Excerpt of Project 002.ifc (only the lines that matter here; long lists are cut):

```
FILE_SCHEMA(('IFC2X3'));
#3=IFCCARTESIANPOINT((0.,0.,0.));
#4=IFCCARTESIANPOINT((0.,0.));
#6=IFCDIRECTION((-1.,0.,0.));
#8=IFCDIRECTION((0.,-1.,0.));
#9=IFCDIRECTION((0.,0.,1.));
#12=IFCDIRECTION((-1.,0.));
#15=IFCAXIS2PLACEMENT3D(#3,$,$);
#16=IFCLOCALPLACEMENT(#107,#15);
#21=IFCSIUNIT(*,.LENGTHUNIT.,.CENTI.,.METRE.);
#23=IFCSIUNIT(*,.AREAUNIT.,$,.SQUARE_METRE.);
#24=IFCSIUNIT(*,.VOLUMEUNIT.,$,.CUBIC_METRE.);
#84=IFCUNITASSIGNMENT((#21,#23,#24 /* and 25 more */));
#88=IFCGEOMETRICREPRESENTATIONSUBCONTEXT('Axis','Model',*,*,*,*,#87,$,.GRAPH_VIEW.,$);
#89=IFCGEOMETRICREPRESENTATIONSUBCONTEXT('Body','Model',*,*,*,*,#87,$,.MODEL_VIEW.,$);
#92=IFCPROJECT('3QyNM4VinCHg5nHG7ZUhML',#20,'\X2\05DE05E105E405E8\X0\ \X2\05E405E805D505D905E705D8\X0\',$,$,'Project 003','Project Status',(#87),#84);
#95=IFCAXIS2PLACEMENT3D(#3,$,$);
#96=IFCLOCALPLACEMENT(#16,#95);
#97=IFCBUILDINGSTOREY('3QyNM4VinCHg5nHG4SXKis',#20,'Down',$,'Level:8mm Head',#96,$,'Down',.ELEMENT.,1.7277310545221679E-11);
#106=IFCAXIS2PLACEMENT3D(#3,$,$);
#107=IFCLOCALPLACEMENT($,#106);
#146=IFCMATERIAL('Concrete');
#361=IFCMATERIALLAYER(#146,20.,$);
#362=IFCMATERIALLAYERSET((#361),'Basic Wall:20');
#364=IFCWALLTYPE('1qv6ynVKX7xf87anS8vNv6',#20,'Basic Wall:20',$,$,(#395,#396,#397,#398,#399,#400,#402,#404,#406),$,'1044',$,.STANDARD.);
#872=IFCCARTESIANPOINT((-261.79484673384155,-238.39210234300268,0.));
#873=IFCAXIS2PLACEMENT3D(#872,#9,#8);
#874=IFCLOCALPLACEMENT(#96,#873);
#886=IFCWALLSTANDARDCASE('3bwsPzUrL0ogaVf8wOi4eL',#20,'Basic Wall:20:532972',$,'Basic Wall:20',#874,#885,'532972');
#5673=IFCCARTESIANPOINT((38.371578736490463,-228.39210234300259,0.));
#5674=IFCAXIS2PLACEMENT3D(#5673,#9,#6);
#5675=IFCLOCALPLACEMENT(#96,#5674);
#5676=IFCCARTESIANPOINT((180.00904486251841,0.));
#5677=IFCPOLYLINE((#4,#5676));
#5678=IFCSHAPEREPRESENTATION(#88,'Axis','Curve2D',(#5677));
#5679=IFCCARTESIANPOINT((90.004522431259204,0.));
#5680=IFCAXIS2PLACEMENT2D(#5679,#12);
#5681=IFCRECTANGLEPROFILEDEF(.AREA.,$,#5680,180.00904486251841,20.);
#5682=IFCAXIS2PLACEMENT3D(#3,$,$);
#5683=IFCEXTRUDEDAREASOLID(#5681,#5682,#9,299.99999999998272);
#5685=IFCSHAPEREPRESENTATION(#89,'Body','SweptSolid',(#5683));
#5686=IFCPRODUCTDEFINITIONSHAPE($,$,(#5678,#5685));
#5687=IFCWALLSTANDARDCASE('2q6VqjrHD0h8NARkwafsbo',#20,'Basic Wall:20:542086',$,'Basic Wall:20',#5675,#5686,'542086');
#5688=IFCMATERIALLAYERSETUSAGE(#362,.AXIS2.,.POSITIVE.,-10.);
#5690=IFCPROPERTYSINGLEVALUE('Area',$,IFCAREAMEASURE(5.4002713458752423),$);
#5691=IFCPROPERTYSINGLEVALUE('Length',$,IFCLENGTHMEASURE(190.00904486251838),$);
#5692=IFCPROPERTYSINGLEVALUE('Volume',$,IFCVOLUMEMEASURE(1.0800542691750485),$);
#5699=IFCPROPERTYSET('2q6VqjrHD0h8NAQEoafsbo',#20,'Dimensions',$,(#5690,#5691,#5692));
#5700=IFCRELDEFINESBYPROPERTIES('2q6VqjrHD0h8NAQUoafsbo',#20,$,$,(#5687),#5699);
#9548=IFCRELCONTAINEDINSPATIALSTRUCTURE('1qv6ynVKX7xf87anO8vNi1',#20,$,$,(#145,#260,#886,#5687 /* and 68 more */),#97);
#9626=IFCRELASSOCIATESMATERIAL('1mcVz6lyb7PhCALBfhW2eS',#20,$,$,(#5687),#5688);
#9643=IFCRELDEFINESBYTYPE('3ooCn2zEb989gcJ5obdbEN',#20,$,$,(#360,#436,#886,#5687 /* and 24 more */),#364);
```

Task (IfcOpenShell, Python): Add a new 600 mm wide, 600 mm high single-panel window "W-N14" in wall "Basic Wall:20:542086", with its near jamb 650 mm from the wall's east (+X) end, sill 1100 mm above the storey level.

```python
import numpy as np
import ifcopenshell
import ifcopenshell.api.feature
import ifcopenshell.api.geometry
import ifcopenshell.api.pset
import ifcopenshell.api.root
import ifcopenshell.api.spatial
import ifcopenshell.api.type
import ifcopenshell.geom
import ifcopenshell.util.element
import ifcopenshell.util.placement
import ifcopenshell.util.representation
import ifcopenshell.util.shape
import ifcopenshell.util.unit

model = ifcopenshell.open("Project 002.ifc")
unit_scale = ifcopenshell.util.unit.calculate_unit_scale(model)
area_scale = ifcopenshell.util.unit.calculate_unit_scale(model, "AREAUNIT")
volume_scale = ifcopenshell.util.unit.calculate_unit_scale(model, "VOLUMEUNIT")
settings = ifcopenshell.geom.settings()


def volume(element):
    """Net volume in cubic metres, openings subtracted."""
    shape = ifcopenshell.geom.create_shape(settings, element)
    return ifcopenshell.util.shape.get_volume(shape.geometry)


wall = model.by_guid("2q6VqjrHD0h8NARkwafsbo")
storey = ifcopenshell.util.element.get_container(wall, ifc_class="IfcBuildingStorey")
context = ifcopenshell.util.representation.get_context(model, "Model", "Body", "MODEL_VIEW")
before = volume(wall)

width, height, from_end, sill = 0.6, 0.6, 0.65, 1.1  # metres

# The wall runs along its own X axis, and the end named is its -X end.
wall_shape = ifcopenshell.geom.create_shape(settings, wall)
x, y, z = ifcopenshell.util.shape.get_vertices(wall_shape.geometry).T
start = x.min() + from_end
face, thickness = float(y.min()), float(y.max() - y.min())
wall_matrix = ifcopenshell.util.placement.get_local_placement(wall.ObjectPlacement)
level = ifcopenshell.util.placement.get_local_placement(storey.ObjectPlacement)[2, 3]


def in_wall(x, y):
    """Placement at x, y metres in the wall's axes, at sill height."""
    matrix = wall_matrix.copy()
    matrix[:, 3] = wall_matrix @ np.array([x / unit_scale, y / unit_scale, 0.0, 1.0])
    matrix[2, 3] = level + sill / unit_scale
    return matrix


# Opening: a box that overshoots both wall faces by 50 mm.
opening = ifcopenshell.api.root.create_entity(model, ifc_class="IfcOpeningElement")
box = ifcopenshell.api.geometry.add_wall_representation(
    model, context=context, length=width, height=height, thickness=thickness + 0.1
)
ifcopenshell.api.geometry.assign_representation(model, product=opening, representation=box)
ifcopenshell.api.geometry.edit_object_placement(model, product=opening, matrix=in_wall(start, face - 0.05), is_si=False)
ifcopenshell.api.feature.add_feature(model, feature=opening, element=wall)

window = ifcopenshell.api.root.create_entity(model, ifc_class="IfcWindow", name="W-N14")
window.OverallWidth, window.OverallHeight = width / unit_scale, height / unit_scale
body = ifcopenshell.api.geometry.add_window_representation(
    model,
    context=context,
    overall_width=window.OverallWidth,
    overall_height=window.OverallHeight,
    partition_type="SINGLE_PANEL",
)
ifcopenshell.api.geometry.assign_representation(model, product=window, representation=body)
ifcopenshell.api.spatial.assign_container(model, products=[window], relating_structure=storey)
fills = ifcopenshell.api.feature.add_filling(model, opening=opening, element=window)
fills.OwnerHistory = window.OwnerHistory  # required in IFC2X3

# IFC2X3 keeps the operation on the window style.
style = ifcopenshell.api.root.create_entity(model, ifc_class="IfcWindowStyle", name="W-N14")
style.OperationType, style.ConstructionType = "SINGLE_PANEL", "NOTDEFINED"
style.ParameterTakesPrecedence = style.Sizeable = False
ifcopenshell.api.type.assign_type(model, related_objects=[window], relating_type=style)

# Centre the window in the wall's thickness.
ifcopenshell.api.geometry.edit_object_placement(model, product=window, matrix=in_wall(start, face), is_si=False)
window_shape = ifcopenshell.geom.create_shape(settings, window)
depth = ifcopenshell.util.shape.get_vertices(window_shape.geometry)[:, 1]
offset = face + thickness / 2 - (depth.min() + depth.max()) / 2
ifcopenshell.api.geometry.edit_object_placement(model, product=window, matrix=in_wall(start, offset), is_si=False)

after = volume(wall)

# Update the wall's stored quantities.
pset = model.by_id(ifcopenshell.util.element.get_pset(wall, "Dimensions", should_inherit=False)["id"])
ifcopenshell.api.pset.edit_pset(model, pset=pset, properties={
    "Area": model.create_entity("IfcAreaMeasure", after / thickness / area_scale),
    "Volume": model.create_entity("IfcVolumeMeasure", after / volume_scale),
})

print(f"wall volume {before:.3f} -> {after:.3f} m3")

model.write("Project 002-out.ifc")
```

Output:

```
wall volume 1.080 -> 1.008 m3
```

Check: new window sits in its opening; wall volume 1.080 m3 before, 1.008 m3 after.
